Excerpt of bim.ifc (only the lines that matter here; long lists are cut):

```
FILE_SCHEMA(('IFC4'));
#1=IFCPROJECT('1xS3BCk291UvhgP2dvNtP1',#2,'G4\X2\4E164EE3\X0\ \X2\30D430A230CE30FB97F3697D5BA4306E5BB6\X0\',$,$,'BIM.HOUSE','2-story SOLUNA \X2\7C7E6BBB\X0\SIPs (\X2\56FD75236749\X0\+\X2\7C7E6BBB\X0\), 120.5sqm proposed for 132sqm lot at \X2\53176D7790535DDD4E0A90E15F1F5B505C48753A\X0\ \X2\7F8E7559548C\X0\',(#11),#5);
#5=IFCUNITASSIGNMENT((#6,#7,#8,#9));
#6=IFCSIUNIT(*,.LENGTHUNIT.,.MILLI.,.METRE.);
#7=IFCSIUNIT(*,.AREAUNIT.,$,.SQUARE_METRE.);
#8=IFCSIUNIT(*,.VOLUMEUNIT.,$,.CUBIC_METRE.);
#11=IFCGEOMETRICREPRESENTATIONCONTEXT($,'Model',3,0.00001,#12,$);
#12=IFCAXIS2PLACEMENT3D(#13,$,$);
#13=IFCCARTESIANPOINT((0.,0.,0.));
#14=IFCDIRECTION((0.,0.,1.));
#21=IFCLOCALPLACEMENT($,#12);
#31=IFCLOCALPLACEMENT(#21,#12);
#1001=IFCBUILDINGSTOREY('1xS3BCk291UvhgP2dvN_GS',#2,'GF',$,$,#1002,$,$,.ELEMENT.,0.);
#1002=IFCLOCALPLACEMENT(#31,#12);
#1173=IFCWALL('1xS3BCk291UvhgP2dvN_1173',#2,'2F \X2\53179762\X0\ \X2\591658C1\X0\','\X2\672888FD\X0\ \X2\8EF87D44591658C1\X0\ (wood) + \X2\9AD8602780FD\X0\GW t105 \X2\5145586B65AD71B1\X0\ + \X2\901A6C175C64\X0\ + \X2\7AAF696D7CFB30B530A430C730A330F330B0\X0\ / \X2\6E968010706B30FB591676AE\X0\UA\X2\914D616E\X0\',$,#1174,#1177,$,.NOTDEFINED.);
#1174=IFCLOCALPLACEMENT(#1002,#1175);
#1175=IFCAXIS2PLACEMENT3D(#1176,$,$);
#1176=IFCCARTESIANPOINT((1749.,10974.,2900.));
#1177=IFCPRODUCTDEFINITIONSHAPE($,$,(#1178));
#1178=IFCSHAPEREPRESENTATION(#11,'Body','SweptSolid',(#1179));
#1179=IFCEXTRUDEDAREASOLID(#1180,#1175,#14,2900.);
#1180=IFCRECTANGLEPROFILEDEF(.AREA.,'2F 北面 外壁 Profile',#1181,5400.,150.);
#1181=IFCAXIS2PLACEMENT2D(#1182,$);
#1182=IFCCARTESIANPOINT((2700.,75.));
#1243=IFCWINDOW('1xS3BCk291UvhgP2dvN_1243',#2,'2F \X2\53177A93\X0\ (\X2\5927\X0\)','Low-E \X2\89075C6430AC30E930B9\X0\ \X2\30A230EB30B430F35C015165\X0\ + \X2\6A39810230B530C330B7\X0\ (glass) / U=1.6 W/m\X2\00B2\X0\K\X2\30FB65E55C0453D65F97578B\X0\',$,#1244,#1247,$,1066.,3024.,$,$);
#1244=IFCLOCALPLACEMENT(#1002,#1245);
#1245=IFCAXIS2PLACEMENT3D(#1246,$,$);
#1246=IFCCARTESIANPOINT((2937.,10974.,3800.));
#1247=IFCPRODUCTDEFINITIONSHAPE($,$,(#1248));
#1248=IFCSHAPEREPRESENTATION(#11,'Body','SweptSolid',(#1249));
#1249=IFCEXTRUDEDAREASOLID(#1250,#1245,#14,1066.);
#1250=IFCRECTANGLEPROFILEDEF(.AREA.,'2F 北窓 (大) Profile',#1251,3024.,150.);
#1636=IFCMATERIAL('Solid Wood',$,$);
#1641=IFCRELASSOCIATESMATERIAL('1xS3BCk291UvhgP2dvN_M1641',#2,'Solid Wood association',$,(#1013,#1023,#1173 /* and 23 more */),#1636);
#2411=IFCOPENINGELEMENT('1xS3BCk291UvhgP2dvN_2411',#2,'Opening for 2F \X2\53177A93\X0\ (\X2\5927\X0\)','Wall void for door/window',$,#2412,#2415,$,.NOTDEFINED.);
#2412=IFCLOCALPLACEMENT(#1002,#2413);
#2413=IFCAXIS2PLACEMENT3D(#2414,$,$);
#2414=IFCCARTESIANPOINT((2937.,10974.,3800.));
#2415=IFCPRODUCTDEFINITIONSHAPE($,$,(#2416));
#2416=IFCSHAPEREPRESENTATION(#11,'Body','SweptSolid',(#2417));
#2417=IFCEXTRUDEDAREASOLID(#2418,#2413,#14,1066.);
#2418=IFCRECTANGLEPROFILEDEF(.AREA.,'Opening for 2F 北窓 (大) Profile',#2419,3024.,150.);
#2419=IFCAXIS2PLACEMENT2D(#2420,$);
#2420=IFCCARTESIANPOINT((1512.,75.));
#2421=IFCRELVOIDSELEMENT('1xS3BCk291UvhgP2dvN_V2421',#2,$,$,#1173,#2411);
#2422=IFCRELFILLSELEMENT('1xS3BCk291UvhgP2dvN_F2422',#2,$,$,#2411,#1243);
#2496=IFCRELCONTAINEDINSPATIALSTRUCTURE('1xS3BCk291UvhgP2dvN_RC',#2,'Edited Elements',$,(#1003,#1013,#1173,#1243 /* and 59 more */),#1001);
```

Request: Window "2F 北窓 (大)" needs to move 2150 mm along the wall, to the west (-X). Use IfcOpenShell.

```python
import ifcopenshell
import ifcopenshell.api.geometry
import ifcopenshell.util.placement

model = ifcopenshell.open("bim.ifc")

window = model.by_guid("1xS3BCk291UvhgP2dvN_1243")
opening = window.FillsVoids[0].RelatingOpeningElement
wall = opening.VoidsElements[0].RelatingBuildingElement

wall_matrix = ifcopenshell.util.placement.get_local_placement(wall.ObjectPlacement)
shift = wall_matrix[:3, 0] * -2150.0
before = ifcopenshell.util.placement.get_local_placement(window.ObjectPlacement)[:3, 3].copy()

# The window is not placed relative to its opening, so move both.
for product in (opening, window):
    matrix = ifcopenshell.util.placement.get_local_placement(product.ObjectPlacement)
    matrix[:3, 3] += shift
    ifcopenshell.api.geometry.edit_object_placement(model, product=product, matrix=matrix, is_si=False)

after = ifcopenshell.util.placement.get_local_placement(window.ObjectPlacement)[:3, 3]
print("window moved by", (after - before).round(3) + 0.0)

model.write("bim_rev.ifc")
```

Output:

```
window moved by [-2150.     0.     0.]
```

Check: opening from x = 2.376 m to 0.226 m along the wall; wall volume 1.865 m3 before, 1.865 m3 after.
